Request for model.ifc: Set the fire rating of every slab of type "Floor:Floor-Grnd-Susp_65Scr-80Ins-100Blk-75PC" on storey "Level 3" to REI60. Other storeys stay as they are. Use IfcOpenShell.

First a look at what the model holds.

```python
import ifcopenshell
import ifcopenshell.util.element

model = ifcopenshell.open("model.ifc")
print(model.schema)
storey = next(s for s in model.by_type("IfcBuildingStorey") if s.Name == "Level 3")
slabs = [e for e in ifcopenshell.util.element.get_decomposition(storey) if e.is_a("IfcSlab")]
seen = {}
for e in slabs:
    element_type = ifcopenshell.util.element.get_type(e)
    key = (element_type.Name if element_type != e and element_type else None, ifcopenshell.util.element.get_pset(e, "Pset_SlabCommon", "FireRating"))
    seen[key] = seen.get(key, 0) + 1
for (name, value), count in sorted(seen.items(), key=str):
    print(count, "x", name, "|", value)
```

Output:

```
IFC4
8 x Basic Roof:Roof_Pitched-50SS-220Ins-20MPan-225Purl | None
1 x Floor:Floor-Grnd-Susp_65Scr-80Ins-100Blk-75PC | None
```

```python
import ifcopenshell
import ifcopenshell.api.pset
import ifcopenshell.util.element

model = ifcopenshell.open("model.ifc")

storey = next(s for s in model.by_type("IfcBuildingStorey") if s.Name == "Level 3")
slabs = [e for e in ifcopenshell.util.element.get_decomposition(storey) if e.is_a("IfcSlab")]

count = 0
for e in slabs:
    element_type = ifcopenshell.util.element.get_type(e)
    if element_type in (None, e) or element_type.Name != "Floor:Floor-Grnd-Susp_65Scr-80Ins-100Blk-75PC":
        continue
    # add_pset returns the element's existing set when there is one.
    pset = ifcopenshell.api.pset.add_pset(model, product=e, name="Pset_SlabCommon")
    ifcopenshell.api.pset.edit_pset(model, pset=pset, properties={"FireRating": "REI60"})
    count += 1

print(count, "slabs updated")

model.write("model_edited.ifc")
```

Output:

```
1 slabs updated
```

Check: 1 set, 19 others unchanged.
